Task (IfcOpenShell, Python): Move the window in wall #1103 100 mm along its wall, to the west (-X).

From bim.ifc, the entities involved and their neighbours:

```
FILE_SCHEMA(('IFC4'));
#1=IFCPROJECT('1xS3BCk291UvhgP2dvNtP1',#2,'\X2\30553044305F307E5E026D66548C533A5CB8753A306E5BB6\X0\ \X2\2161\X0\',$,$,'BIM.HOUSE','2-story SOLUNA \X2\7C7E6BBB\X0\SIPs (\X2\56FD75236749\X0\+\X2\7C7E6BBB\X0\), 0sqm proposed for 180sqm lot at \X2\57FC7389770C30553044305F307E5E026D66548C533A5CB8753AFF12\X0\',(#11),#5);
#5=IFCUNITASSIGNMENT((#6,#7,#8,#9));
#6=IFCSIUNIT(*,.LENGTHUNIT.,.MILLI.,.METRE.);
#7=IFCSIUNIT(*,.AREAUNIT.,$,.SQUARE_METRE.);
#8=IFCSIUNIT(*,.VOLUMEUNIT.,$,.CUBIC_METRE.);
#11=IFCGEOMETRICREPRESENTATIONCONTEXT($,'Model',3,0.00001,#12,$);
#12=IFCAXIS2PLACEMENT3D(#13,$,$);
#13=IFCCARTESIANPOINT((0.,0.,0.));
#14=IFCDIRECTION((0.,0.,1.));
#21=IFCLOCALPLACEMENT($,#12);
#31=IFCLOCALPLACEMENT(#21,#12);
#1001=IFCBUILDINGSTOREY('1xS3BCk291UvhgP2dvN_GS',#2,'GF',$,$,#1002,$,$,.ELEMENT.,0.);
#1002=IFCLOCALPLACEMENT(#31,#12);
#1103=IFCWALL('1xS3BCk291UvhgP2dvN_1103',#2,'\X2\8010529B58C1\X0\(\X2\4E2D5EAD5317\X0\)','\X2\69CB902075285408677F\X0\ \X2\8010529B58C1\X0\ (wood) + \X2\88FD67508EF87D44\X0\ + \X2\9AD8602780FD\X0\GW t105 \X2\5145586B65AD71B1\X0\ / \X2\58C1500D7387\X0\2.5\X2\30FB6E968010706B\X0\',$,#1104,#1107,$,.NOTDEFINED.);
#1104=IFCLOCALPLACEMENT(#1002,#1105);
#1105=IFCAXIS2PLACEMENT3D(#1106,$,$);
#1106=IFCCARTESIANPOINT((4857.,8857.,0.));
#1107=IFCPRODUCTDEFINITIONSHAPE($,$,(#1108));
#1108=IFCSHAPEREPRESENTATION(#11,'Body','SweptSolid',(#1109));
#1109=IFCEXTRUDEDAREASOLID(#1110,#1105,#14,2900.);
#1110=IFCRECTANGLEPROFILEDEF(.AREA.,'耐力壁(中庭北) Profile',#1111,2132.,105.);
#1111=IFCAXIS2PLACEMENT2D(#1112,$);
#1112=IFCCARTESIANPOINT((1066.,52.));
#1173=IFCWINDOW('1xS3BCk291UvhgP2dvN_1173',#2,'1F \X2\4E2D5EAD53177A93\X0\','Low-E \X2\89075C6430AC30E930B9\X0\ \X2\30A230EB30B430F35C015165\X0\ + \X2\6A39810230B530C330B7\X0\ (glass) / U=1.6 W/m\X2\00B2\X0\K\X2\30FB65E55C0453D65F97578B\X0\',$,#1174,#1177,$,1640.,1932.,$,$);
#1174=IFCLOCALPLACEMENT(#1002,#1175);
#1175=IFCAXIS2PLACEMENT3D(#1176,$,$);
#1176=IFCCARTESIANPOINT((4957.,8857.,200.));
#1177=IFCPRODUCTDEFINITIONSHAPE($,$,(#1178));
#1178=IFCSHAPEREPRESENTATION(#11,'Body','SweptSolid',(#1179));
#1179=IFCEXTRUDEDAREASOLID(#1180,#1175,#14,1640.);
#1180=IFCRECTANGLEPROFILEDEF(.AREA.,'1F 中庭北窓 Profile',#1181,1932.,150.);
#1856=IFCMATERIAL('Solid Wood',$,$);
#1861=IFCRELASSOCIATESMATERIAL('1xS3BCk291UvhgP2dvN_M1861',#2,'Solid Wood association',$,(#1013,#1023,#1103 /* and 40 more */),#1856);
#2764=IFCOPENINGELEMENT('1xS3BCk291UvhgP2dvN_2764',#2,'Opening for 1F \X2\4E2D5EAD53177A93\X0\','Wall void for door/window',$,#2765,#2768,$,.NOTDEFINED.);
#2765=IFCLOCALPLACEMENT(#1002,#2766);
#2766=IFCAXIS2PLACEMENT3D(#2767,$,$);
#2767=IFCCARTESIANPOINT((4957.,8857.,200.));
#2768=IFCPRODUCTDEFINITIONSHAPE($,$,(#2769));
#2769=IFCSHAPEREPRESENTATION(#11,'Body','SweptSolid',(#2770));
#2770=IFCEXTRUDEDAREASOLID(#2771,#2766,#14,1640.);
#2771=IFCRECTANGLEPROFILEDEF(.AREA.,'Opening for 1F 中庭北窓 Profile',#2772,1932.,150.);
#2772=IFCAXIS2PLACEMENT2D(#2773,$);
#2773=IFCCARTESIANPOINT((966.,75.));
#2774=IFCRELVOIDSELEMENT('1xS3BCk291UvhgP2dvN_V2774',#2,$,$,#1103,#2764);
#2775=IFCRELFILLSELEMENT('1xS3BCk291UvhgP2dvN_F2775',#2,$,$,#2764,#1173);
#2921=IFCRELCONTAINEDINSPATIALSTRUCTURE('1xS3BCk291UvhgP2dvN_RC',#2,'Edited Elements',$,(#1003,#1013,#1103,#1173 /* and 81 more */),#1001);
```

```python
import ifcopenshell
import ifcopenshell.api.geometry
import ifcopenshell.util.placement
import ifcopenshell.util.unit

model = ifcopenshell.open("bim.ifc")
unit_scale = ifcopenshell.util.unit.calculate_unit_scale(model)

window = model.by_guid("1xS3BCk291UvhgP2dvN_1173")
opening = window.FillsVoids[0].RelatingOpeningElement
wall = opening.VoidsElements[0].RelatingBuildingElement

wall_matrix = ifcopenshell.util.placement.get_local_placement(wall.ObjectPlacement)
shift = wall_matrix[:3, 0] * -0.1 / unit_scale
before = ifcopenshell.util.placement.get_local_placement(window.ObjectPlacement)[:3, 3].copy()

# The window is not placed relative to its opening, so move both.
for product in (opening, window):
    matrix = ifcopenshell.util.placement.get_local_placement(product.ObjectPlacement)
    matrix[:3, 3] += shift
    ifcopenshell.api.geometry.edit_object_placement(model, product=product, matrix=matrix, is_si=False)

after = ifcopenshell.util.placement.get_local_placement(window.ObjectPlacement)[:3, 3]
print("window moved by", (after - before).round(3) + 0.0)

model.write("bim_edited.ifc")
```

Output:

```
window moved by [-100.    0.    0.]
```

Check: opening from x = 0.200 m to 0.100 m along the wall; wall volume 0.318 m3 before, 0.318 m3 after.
